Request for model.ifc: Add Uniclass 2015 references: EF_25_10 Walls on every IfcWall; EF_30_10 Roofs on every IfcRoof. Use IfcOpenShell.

First a look at what the model holds.

```python
import ifcopenshell

model = ifcopenshell.open("model.ifc")
print(model.schema)
print("classifications:", [c.Name for c in model.by_type("IfcClassification")])
for ifc_class in ("IfcDoor", "IfcRoof", "IfcStair", "IfcWall", "IfcWindow"):
    print(ifc_class, len(model.by_type(ifc_class)))
```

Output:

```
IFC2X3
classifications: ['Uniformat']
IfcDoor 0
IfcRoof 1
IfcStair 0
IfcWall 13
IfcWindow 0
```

```python
import ifcopenshell
import ifcopenshell.api.classification

model = ifcopenshell.open("model.ifc")

# IFC2X3 requires Source and Edition and has no link from the project to the system.
system = model.create_entity("IfcClassification", Source="NBS", Edition="2015", Name="Uniclass 2015")

codes = {
    "IfcWall": ("EF_25_10", "Walls"),
    "IfcRoof": ("EF_30_10", "Roofs"),
}
for ifc_class, (code, name) in codes.items():
    products = model.by_type(ifc_class)
    ifcopenshell.api.classification.add_reference(
        model, products=products, classification=system, identification=code, name=name
    )
    print(code, len(products))

model.write("model_rev.ifc")
```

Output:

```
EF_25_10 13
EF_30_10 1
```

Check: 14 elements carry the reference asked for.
